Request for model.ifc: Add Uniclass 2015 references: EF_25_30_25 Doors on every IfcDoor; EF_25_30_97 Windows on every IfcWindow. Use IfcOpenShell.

First a look at what the model holds.

```python
import ifcopenshell

model = ifcopenshell.open("model.ifc")
print(model.schema)
print("classifications:", [c.Name for c in model.by_type("IfcClassification")])
for ifc_class in ("IfcDoor", "IfcRoof", "IfcStair", "IfcWall", "IfcWindow"):
    print(ifc_class, len(model.by_type(ifc_class)))
```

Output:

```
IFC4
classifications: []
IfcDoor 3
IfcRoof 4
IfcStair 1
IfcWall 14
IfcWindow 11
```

```python
import ifcopenshell
import ifcopenshell.api.classification

model = ifcopenshell.open("model.ifc")

system = ifcopenshell.api.classification.add_classification(model, classification="Uniclass 2015")

codes = {
    "IfcDoor": ("EF_25_30_25", "Doors"),
    "IfcWindow": ("EF_25_30_97", "Windows"),
}
for ifc_class, (code, name) in codes.items():
    products = model.by_type(ifc_class)
    ifcopenshell.api.classification.add_reference(
        model, products=products, classification=system, identification=code, name=name
    )
    print(code, len(products))

model.write("model_edited.ifc")
```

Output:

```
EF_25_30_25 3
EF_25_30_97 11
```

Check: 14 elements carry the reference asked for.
